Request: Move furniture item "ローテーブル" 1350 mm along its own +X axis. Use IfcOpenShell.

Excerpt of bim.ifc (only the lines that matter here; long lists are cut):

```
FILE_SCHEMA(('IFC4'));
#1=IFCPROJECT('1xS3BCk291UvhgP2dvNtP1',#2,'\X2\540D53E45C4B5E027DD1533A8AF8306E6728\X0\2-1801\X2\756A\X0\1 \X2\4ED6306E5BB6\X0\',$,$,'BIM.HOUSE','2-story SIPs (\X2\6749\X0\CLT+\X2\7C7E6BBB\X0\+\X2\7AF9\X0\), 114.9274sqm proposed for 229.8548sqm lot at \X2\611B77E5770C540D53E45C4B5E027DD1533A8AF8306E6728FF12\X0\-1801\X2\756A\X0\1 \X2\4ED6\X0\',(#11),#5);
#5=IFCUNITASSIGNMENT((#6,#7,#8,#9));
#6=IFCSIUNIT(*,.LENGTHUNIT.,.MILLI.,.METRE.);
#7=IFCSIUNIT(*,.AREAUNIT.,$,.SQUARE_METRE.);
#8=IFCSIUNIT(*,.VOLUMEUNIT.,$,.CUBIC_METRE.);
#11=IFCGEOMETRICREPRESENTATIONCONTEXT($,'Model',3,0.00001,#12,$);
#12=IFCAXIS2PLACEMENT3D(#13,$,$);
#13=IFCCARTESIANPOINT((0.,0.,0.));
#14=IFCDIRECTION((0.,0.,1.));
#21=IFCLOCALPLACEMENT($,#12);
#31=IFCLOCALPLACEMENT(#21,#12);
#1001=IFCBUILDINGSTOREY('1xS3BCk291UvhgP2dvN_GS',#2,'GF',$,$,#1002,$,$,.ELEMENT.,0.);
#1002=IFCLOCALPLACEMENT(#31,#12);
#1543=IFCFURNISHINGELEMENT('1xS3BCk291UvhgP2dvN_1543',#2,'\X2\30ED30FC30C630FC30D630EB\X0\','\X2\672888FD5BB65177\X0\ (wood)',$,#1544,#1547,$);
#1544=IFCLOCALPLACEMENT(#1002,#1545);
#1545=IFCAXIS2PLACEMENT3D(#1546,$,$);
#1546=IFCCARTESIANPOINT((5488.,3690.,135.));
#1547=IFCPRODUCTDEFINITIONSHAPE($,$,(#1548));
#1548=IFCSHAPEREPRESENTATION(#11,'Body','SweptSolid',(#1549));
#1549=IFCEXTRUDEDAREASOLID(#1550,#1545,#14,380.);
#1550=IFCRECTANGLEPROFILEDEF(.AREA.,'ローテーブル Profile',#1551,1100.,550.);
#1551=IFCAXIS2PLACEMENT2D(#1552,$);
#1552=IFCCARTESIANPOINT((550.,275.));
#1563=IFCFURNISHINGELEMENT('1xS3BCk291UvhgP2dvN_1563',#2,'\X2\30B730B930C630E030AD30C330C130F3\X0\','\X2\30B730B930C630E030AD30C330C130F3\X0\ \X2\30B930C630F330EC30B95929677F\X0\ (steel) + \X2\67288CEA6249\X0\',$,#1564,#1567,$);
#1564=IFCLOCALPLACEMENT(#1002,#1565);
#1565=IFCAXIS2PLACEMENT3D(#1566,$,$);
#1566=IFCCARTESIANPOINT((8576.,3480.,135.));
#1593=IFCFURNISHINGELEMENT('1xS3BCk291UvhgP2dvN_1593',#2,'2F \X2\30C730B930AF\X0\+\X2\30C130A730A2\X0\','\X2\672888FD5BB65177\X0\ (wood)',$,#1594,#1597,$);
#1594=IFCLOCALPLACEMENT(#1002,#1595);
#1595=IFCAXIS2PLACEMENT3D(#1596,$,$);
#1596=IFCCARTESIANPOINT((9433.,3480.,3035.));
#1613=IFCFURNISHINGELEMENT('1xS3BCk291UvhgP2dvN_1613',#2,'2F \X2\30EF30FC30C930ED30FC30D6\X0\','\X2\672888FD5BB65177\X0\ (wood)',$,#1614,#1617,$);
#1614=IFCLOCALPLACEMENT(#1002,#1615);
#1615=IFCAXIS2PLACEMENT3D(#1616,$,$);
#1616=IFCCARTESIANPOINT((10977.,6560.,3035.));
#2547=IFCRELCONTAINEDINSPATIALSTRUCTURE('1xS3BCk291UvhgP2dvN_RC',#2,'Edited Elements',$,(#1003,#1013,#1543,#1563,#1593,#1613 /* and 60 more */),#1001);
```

```python
import ifcopenshell
import ifcopenshell.api.geometry
import ifcopenshell.util.placement
import ifcopenshell.util.unit

model = ifcopenshell.open("bim.ifc")
unit_scale = ifcopenshell.util.unit.calculate_unit_scale(model)

item = model.by_guid("1xS3BCk291UvhgP2dvN_1543")
matrix = ifcopenshell.util.placement.get_local_placement(item.ObjectPlacement)
matrix[:3, 3] += matrix[:3, 0] * 1.35 / unit_scale
ifcopenshell.api.geometry.edit_object_placement(model, product=item, matrix=matrix, is_si=False)

print(ifcopenshell.util.placement.get_local_placement(item.ObjectPlacement).round(3) + 0.0)

model.write("bim-out.ifc")
```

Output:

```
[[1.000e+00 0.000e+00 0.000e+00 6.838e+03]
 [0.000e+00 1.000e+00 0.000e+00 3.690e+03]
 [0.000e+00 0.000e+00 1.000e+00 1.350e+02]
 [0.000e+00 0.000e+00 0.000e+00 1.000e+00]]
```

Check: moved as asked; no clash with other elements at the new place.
